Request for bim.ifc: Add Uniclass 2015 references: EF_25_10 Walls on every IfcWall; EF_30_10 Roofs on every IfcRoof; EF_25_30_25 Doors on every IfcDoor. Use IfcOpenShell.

First a look at what the model holds.

```python
import ifcopenshell

model = ifcopenshell.open("bim.ifc")
print(model.schema)
print("classifications:", [c.Name for c in model.by_type("IfcClassification")])
for ifc_class in ("IfcDoor", "IfcRoof", "IfcStair", "IfcWall", "IfcWindow"):
    print(ifc_class, len(model.by_type(ifc_class)))
```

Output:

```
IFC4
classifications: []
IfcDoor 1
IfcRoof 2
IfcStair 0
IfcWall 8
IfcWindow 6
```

```python
import ifcopenshell
import ifcopenshell.api.classification

model = ifcopenshell.open("bim.ifc")

system = ifcopenshell.api.classification.add_classification(model, classification="Uniclass 2015")

codes = {
    "IfcWall": ("EF_25_10", "Walls"),
    "IfcRoof": ("EF_30_10", "Roofs"),
    "IfcDoor": ("EF_25_30_25", "Doors"),
}
for ifc_class, (code, name) in codes.items():
    products = model.by_type(ifc_class)
    ifcopenshell.api.classification.add_reference(
        model, products=products, classification=system, identification=code, name=name
    )
    print(code, len(products))

model.write("bim_v2.ifc")
```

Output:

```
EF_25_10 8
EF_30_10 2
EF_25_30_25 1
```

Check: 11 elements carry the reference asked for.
